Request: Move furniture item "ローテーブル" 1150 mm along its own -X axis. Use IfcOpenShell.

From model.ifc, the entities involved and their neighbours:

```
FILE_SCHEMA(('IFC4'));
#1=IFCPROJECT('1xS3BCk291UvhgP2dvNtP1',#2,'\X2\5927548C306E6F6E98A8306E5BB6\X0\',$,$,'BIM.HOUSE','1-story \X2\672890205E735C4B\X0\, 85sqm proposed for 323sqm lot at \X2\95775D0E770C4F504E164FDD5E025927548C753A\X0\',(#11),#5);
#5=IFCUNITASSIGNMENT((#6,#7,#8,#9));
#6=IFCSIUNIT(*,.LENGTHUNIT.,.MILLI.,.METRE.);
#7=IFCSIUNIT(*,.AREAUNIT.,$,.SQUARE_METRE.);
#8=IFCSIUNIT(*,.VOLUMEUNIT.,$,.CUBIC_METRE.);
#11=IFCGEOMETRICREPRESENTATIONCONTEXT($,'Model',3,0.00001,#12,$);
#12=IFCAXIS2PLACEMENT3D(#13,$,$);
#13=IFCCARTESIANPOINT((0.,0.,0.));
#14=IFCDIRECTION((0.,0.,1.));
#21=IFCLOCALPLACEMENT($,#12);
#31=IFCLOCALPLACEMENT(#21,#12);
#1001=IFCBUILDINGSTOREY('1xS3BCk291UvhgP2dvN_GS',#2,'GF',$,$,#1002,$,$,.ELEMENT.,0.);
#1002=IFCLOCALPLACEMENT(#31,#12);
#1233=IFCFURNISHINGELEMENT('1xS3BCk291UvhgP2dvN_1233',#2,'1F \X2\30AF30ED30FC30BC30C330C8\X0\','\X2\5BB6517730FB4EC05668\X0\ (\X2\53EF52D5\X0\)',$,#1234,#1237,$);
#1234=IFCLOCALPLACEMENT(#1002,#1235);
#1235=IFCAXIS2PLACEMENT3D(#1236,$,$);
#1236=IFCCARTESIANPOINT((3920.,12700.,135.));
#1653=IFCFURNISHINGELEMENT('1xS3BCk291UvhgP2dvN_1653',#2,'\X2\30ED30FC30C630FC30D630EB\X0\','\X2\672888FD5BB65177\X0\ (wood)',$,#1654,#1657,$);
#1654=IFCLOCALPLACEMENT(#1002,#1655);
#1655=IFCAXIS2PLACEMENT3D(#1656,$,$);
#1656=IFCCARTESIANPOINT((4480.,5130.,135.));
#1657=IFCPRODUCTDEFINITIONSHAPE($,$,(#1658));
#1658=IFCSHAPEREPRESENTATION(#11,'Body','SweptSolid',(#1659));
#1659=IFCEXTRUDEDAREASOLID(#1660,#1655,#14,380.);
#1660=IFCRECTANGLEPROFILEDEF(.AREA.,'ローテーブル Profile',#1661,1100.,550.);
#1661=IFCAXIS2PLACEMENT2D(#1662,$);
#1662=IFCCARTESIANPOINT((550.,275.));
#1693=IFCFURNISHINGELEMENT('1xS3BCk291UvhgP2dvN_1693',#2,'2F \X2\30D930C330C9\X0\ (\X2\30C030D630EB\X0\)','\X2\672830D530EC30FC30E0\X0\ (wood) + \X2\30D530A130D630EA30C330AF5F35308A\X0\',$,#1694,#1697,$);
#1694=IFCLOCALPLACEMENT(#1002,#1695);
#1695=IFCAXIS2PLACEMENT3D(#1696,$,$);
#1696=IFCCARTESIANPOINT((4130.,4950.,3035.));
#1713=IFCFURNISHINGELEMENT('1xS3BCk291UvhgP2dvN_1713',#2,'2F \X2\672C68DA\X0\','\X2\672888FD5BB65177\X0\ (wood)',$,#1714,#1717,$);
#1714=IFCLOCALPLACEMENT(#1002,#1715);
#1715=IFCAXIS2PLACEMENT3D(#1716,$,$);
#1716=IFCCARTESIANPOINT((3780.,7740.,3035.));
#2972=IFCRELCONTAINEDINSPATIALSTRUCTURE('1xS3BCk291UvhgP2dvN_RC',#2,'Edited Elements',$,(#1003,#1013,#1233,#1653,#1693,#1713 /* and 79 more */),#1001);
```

```python
import ifcopenshell
import ifcopenshell.api.geometry
import ifcopenshell.util.placement
import ifcopenshell.util.unit

model = ifcopenshell.open("model.ifc")
unit_scale = ifcopenshell.util.unit.calculate_unit_scale(model)

item = model.by_guid("1xS3BCk291UvhgP2dvN_1653")
matrix = ifcopenshell.util.placement.get_local_placement(item.ObjectPlacement)
matrix[:3, 3] -= matrix[:3, 0] * 1.15 / unit_scale
ifcopenshell.api.geometry.edit_object_placement(model, product=item, matrix=matrix, is_si=False)

print(ifcopenshell.util.placement.get_local_placement(item.ObjectPlacement).round(3) + 0.0)

model.write("model_updated.ifc")
```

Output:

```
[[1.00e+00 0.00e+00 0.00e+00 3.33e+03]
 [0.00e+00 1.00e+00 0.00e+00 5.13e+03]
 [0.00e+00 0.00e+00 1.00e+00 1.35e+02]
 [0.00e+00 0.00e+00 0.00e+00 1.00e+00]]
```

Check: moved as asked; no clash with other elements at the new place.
